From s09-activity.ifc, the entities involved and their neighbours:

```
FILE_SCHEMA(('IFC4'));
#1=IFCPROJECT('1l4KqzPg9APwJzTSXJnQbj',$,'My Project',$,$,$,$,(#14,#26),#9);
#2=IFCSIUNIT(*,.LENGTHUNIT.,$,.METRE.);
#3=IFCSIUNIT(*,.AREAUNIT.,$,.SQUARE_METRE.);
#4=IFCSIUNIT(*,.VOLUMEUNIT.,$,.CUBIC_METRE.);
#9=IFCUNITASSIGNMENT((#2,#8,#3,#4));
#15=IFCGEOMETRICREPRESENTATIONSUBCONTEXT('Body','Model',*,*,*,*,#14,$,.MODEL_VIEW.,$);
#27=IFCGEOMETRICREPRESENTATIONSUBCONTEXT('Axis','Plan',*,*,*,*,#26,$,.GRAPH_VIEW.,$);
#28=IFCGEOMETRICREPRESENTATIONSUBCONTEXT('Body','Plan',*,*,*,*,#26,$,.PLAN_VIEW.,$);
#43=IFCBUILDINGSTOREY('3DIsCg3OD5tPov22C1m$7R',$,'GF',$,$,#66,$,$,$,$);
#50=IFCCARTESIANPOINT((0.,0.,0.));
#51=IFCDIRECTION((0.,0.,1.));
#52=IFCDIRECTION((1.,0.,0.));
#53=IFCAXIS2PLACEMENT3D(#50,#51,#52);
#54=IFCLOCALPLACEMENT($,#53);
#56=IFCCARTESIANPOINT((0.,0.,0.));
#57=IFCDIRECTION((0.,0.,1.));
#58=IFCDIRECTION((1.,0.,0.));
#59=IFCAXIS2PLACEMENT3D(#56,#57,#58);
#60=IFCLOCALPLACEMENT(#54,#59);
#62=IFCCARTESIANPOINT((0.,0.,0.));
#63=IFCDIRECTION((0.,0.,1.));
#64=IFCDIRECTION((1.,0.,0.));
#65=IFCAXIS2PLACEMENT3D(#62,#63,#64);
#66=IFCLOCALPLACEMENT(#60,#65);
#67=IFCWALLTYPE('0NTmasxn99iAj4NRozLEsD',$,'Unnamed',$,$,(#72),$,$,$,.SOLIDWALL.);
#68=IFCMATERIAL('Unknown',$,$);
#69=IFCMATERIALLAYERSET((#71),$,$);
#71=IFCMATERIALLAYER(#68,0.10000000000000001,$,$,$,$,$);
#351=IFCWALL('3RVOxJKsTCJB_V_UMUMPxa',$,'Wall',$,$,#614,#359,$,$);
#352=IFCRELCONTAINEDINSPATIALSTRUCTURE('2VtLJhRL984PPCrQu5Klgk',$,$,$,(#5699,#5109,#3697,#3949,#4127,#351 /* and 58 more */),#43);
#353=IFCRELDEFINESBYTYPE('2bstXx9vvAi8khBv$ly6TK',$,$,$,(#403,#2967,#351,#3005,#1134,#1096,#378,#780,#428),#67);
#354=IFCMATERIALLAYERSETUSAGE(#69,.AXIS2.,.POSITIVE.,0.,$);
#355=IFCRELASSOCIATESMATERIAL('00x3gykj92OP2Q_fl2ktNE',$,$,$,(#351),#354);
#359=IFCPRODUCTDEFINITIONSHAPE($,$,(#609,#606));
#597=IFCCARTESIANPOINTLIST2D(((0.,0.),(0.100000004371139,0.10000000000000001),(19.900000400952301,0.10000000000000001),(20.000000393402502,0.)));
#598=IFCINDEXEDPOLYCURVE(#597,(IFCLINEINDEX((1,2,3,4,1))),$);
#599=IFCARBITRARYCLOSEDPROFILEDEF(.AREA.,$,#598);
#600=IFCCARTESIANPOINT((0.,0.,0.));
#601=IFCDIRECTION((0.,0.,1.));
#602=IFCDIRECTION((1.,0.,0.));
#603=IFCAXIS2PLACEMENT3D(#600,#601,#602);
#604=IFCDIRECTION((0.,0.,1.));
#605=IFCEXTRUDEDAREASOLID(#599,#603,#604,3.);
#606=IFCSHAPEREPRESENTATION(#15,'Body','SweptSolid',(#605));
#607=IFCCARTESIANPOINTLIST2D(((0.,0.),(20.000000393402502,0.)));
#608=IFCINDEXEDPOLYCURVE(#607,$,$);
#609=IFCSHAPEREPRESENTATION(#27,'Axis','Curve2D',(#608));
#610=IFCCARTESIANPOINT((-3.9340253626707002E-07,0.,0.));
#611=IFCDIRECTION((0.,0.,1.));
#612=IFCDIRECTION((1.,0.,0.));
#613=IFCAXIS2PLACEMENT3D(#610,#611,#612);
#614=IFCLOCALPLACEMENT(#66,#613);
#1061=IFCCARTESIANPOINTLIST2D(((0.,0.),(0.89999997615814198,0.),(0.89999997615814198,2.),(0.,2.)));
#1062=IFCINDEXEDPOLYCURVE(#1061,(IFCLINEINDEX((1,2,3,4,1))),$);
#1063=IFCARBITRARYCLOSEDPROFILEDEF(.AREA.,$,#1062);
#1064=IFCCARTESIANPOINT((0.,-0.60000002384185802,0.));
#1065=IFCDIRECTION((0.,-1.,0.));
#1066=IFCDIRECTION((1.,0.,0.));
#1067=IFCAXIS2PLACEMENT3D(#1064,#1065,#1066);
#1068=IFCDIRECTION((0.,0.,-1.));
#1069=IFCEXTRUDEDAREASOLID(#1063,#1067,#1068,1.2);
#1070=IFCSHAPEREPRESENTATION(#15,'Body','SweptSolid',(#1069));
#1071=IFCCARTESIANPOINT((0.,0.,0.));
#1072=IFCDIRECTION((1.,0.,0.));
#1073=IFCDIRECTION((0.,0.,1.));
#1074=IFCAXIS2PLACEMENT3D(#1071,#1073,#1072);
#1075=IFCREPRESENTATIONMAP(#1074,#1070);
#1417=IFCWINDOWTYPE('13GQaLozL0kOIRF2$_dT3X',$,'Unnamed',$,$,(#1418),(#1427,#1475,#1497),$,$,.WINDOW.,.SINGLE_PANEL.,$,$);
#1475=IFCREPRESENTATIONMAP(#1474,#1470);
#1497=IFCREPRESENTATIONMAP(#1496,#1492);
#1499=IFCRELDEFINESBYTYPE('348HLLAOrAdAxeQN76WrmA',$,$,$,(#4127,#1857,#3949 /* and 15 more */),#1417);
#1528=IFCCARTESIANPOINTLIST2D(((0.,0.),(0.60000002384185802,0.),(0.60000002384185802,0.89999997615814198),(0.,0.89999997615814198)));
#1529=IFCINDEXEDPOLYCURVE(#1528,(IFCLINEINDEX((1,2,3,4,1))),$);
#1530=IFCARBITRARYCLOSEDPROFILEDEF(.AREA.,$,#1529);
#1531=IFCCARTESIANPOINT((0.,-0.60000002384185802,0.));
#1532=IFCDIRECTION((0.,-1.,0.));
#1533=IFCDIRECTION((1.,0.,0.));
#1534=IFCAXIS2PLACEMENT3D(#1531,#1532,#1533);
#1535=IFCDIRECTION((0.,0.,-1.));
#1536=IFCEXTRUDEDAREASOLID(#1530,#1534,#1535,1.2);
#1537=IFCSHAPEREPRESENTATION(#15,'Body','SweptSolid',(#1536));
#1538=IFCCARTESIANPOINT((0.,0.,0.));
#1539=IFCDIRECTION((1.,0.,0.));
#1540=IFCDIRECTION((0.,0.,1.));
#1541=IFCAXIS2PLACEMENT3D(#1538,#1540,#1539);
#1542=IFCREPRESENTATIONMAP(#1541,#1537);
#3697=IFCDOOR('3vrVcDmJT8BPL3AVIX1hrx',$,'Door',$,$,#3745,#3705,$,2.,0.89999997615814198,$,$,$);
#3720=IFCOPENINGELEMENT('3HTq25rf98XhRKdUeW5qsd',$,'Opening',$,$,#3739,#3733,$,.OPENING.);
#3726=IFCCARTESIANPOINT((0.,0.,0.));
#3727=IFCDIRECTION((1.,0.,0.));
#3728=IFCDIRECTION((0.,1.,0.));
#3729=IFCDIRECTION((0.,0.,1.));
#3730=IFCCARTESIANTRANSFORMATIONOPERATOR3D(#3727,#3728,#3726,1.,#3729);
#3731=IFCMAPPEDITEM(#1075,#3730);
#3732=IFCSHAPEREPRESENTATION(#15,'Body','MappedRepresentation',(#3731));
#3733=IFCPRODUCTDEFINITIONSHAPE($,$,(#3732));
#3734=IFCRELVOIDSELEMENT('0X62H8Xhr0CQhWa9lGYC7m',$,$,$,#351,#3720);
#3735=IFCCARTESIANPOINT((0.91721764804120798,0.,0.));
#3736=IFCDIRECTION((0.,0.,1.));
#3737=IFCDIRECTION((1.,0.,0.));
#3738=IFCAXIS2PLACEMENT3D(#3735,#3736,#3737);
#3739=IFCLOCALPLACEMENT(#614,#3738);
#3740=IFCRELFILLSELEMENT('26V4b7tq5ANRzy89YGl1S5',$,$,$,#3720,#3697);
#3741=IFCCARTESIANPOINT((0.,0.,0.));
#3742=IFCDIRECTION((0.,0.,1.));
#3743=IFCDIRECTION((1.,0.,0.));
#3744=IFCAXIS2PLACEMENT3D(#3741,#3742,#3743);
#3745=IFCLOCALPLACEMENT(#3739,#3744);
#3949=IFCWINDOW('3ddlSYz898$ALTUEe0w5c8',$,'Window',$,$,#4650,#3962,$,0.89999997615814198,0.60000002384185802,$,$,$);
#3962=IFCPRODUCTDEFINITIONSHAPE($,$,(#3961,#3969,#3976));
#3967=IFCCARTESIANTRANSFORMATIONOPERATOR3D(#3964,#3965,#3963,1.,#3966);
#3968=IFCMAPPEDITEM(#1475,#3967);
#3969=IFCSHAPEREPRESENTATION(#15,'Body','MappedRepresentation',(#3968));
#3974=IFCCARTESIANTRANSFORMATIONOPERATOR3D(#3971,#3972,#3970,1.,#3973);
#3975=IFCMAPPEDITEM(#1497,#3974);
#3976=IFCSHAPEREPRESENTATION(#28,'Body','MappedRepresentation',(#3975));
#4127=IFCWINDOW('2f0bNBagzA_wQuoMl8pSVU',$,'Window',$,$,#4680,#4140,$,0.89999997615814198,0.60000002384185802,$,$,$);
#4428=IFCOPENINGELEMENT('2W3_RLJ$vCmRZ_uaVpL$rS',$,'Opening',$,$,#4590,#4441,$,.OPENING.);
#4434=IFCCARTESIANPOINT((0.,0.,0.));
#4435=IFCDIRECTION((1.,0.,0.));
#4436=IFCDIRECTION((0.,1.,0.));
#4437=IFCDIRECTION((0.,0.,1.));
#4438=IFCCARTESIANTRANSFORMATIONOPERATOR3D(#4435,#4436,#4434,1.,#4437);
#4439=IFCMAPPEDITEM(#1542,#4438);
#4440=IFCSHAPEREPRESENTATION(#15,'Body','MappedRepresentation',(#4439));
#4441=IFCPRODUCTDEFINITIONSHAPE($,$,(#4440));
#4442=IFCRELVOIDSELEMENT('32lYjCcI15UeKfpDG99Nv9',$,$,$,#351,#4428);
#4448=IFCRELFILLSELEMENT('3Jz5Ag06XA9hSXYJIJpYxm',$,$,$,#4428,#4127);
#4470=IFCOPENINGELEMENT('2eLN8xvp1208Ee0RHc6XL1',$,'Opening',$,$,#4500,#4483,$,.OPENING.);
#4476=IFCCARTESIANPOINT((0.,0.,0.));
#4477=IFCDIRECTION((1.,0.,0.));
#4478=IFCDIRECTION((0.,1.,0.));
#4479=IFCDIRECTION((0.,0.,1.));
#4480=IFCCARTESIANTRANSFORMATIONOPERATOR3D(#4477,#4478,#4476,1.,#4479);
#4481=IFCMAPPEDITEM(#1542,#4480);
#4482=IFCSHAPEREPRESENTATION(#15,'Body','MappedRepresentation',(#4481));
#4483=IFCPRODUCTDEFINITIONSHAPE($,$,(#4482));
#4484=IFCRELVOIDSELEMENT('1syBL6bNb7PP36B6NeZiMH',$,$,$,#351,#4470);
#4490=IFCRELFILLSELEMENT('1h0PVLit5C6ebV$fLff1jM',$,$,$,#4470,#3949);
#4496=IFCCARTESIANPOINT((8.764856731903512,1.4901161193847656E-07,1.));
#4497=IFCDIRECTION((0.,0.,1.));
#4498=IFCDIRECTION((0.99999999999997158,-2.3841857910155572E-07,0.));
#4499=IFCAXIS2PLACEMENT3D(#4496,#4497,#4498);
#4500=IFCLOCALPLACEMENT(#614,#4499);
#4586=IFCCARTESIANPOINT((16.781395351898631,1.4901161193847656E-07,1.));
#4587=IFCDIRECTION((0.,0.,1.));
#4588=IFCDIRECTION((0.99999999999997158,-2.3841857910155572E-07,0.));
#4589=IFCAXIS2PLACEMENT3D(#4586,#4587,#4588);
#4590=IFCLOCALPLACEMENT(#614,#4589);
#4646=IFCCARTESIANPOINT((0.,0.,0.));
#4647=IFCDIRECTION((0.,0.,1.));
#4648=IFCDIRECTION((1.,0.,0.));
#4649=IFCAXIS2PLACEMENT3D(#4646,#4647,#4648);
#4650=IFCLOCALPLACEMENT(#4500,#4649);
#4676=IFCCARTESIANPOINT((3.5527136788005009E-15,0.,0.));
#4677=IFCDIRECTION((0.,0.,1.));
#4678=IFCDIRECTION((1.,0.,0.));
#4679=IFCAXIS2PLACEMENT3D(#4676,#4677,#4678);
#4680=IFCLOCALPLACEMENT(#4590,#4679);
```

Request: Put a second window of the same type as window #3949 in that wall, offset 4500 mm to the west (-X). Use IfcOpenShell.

```python
import ifcopenshell
import ifcopenshell.api.feature
import ifcopenshell.api.geometry
import ifcopenshell.api.root
import ifcopenshell.geom
import ifcopenshell.util.element
import ifcopenshell.util.placement
import ifcopenshell.util.shape
import ifcopenshell.util.unit

model = ifcopenshell.open("s09-activity.ifc")
unit_scale = ifcopenshell.util.unit.calculate_unit_scale(model)
settings = ifcopenshell.geom.settings()


def volume(element):
    """Net volume in cubic metres, openings subtracted."""
    shape = ifcopenshell.geom.create_shape(settings, element)
    return ifcopenshell.util.shape.get_volume(shape.geometry)


window = model.by_guid("3ddlSYz898$ALTUEe0w5c8")
opening = window.FillsVoids[0].RelatingOpeningElement
wall = opening.VoidsElements[0].RelatingBuildingElement
before = volume(wall)
shift = ifcopenshell.util.placement.get_local_placement(wall.ObjectPlacement)[:3, 0] * -4.5 / unit_scale

# copy_class copies the void relationship, type, container and properties, but no geometry.
new_opening = ifcopenshell.api.root.copy_class(model, product=opening)
new_opening.Representation = ifcopenshell.util.element.copy_deep(
    model, opening.Representation, exclude=["IfcGeometricRepresentationContext", "IfcRepresentationMap"]
)
new_window = ifcopenshell.api.root.copy_class(model, product=window)
new_window.Representation = ifcopenshell.util.element.copy_deep(
    model, window.Representation, exclude=["IfcGeometricRepresentationContext", "IfcRepresentationMap"]
)
ifcopenshell.api.feature.add_filling(model, opening=new_opening, element=new_window)

for old, new in ((opening, new_opening), (window, new_window)):
    matrix = ifcopenshell.util.placement.get_local_placement(old.ObjectPlacement)
    matrix[:3, 3] += shift
    ifcopenshell.api.geometry.edit_object_placement(model, product=new, matrix=matrix, is_si=False)

after = volume(wall)

print(f"wall volume {before:.3f} -> {after:.3f} m3")

model.write("s09-activity_v2.ifc")
```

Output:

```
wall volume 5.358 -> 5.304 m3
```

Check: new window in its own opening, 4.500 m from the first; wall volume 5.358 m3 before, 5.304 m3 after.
